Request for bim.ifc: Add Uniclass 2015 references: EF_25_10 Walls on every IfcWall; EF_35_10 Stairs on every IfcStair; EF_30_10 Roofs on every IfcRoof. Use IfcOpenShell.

First a look at what the model holds.

```python
import ifcopenshell

model = ifcopenshell.open("bim.ifc")
print(model.schema)
print("classifications:", [c.Name for c in model.by_type("IfcClassification")])
for ifc_class in ("IfcDoor", "IfcRoof", "IfcStair", "IfcWall", "IfcWindow"):
    print(ifc_class, len(model.by_type(ifc_class)))
```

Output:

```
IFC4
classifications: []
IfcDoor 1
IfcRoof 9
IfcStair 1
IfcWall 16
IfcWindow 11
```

```python
import ifcopenshell
import ifcopenshell.api.classification

model = ifcopenshell.open("bim.ifc")

system = ifcopenshell.api.classification.add_classification(model, classification="Uniclass 2015")

codes = {
    "IfcWall": ("EF_25_10", "Walls"),
    "IfcStair": ("EF_35_10", "Stairs"),
    "IfcRoof": ("EF_30_10", "Roofs"),
}
for ifc_class, (code, name) in codes.items():
    products = model.by_type(ifc_class)
    ifcopenshell.api.classification.add_reference(
        model, products=products, classification=system, identification=code, name=name
    )
    print(code, len(products))

model.write("bim-out.ifc")
```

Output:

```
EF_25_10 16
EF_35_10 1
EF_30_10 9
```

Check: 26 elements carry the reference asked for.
